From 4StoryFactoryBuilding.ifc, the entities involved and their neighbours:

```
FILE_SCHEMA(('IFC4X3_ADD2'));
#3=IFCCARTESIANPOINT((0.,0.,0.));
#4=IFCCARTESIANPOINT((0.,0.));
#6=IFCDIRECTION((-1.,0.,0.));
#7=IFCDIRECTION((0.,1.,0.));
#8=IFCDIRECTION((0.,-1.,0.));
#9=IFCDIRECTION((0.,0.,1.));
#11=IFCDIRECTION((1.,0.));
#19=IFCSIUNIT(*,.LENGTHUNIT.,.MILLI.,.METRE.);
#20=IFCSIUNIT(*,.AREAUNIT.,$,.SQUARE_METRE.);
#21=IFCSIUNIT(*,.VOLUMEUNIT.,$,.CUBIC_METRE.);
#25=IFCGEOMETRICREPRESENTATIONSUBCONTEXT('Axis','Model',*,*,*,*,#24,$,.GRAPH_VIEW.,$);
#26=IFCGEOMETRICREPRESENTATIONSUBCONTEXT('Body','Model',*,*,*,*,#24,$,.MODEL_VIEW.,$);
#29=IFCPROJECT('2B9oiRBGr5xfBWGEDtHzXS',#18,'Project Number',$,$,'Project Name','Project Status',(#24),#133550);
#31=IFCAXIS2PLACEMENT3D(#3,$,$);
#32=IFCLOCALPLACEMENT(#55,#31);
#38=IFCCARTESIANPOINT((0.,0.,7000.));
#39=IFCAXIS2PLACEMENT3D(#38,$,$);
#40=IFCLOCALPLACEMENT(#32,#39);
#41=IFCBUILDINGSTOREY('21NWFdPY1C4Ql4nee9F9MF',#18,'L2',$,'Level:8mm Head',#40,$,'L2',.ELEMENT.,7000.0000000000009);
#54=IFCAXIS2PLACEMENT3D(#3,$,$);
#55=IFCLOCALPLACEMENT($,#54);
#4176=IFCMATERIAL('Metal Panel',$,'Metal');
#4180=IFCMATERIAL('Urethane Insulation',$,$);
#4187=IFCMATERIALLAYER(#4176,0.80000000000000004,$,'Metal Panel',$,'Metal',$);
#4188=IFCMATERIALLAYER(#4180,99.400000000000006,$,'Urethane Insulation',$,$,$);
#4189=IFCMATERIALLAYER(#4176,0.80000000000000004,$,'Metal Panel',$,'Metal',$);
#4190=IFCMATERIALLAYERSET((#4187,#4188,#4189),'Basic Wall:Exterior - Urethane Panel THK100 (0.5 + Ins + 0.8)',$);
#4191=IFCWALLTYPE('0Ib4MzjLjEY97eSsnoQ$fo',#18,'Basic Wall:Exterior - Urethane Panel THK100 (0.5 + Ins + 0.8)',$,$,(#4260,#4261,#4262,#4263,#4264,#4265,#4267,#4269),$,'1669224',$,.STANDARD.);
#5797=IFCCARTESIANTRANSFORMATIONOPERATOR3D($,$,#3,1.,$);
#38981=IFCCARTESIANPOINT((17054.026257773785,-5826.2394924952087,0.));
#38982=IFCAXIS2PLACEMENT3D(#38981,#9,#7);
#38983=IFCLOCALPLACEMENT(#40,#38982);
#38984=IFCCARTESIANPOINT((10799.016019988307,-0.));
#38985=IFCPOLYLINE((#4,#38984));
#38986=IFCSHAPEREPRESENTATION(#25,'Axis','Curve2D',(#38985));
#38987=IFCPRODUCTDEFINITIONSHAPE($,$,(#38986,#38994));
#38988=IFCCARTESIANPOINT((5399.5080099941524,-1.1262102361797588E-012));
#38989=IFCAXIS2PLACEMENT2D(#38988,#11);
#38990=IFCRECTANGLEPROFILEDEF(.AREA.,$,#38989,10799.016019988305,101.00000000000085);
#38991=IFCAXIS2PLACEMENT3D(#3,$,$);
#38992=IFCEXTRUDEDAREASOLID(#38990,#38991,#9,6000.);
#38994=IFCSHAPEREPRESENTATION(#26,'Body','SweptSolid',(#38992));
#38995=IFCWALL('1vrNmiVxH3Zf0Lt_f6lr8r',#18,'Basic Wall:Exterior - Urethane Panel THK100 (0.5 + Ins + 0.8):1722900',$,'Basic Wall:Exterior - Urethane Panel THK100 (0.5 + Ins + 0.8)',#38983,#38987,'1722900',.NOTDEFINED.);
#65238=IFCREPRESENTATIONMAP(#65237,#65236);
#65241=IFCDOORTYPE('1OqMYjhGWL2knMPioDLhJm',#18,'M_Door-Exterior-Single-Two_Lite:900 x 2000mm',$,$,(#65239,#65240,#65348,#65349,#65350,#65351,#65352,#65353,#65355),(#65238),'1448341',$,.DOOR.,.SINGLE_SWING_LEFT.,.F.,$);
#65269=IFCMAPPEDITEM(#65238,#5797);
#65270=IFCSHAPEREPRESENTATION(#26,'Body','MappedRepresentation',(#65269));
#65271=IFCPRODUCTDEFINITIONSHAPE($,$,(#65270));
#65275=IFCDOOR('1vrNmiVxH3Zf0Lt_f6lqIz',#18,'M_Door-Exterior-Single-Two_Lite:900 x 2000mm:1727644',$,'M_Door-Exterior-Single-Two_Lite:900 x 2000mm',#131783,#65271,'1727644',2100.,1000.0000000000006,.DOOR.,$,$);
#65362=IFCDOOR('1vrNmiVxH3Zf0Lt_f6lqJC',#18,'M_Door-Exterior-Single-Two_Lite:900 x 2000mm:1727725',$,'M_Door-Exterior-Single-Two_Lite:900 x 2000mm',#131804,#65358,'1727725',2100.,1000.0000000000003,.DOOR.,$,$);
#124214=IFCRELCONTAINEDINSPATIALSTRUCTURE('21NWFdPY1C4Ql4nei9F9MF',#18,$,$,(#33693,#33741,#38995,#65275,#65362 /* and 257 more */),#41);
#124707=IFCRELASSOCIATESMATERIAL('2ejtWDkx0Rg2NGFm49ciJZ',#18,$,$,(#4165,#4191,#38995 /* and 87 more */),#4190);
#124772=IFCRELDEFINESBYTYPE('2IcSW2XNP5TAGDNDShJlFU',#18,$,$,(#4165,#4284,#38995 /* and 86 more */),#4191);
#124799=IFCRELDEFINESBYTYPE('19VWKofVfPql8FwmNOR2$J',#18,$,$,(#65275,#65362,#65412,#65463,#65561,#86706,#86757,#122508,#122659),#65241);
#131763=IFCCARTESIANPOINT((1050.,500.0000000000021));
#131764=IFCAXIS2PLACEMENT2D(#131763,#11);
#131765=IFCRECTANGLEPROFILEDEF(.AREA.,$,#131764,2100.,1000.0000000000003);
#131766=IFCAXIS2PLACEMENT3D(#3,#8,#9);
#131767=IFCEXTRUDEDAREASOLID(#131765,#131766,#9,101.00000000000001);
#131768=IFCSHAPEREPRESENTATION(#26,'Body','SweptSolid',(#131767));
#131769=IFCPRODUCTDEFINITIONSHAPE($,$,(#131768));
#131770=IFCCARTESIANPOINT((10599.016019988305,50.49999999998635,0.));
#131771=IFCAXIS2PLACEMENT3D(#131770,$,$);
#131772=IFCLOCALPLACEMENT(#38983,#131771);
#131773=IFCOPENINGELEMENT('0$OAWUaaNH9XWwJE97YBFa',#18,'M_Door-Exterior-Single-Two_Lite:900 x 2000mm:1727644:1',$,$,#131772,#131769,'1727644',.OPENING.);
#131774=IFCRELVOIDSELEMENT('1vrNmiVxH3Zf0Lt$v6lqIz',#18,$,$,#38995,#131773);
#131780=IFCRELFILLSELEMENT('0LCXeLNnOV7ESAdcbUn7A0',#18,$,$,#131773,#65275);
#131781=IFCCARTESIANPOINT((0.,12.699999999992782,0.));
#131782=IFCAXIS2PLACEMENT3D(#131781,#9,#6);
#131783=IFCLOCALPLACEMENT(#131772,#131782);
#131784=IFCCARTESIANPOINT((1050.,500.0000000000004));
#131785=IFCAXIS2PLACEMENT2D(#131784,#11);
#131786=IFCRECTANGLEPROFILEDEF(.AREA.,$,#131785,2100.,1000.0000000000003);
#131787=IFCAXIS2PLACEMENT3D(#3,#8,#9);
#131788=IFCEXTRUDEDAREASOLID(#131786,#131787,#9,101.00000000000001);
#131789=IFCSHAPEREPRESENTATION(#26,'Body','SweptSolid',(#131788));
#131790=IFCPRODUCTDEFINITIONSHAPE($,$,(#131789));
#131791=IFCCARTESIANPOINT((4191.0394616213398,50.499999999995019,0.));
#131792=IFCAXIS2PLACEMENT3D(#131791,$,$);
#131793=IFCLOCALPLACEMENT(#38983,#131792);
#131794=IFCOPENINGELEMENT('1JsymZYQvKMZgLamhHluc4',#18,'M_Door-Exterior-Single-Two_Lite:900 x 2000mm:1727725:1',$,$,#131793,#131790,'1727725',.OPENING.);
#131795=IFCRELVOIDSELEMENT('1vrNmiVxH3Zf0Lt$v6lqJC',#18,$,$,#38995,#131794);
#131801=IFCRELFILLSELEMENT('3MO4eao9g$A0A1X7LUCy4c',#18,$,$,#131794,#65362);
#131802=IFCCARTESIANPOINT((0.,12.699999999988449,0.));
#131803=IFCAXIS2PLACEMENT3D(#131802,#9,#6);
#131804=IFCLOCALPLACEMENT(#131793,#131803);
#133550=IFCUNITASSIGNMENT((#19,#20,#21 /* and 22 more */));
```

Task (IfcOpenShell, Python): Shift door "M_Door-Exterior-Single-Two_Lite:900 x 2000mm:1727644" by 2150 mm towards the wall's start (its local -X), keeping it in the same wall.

```python
import ifcopenshell
import ifcopenshell.api.geometry
import ifcopenshell.util.placement
import ifcopenshell.util.unit

model = ifcopenshell.open("4StoryFactoryBuilding.ifc")
unit_scale = ifcopenshell.util.unit.calculate_unit_scale(model)

door = model.by_guid("1vrNmiVxH3Zf0Lt_f6lqIz")
opening = door.FillsVoids[0].RelatingOpeningElement
wall = opening.VoidsElements[0].RelatingBuildingElement

wall_matrix = ifcopenshell.util.placement.get_local_placement(wall.ObjectPlacement)
shift = wall_matrix[:3, 0] * -2.15 / unit_scale
before = ifcopenshell.util.placement.get_local_placement(door.ObjectPlacement)[:3, 3].copy()

# The door is placed relative to its opening, so it follows when the opening moves.
matrix = ifcopenshell.util.placement.get_local_placement(opening.ObjectPlacement)
matrix[:3, 3] += shift
ifcopenshell.api.geometry.edit_object_placement(
    model, product=opening, matrix=matrix, is_si=False, should_transform_children=True
)

after = ifcopenshell.util.placement.get_local_placement(door.ObjectPlacement)[:3, 3]
print("door moved by", (after - before).round(3) + 0.0)

model.write("4StoryFactoryBuilding_edited.ifc")
```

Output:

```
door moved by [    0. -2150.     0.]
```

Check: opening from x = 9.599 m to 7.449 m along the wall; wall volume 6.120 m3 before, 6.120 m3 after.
